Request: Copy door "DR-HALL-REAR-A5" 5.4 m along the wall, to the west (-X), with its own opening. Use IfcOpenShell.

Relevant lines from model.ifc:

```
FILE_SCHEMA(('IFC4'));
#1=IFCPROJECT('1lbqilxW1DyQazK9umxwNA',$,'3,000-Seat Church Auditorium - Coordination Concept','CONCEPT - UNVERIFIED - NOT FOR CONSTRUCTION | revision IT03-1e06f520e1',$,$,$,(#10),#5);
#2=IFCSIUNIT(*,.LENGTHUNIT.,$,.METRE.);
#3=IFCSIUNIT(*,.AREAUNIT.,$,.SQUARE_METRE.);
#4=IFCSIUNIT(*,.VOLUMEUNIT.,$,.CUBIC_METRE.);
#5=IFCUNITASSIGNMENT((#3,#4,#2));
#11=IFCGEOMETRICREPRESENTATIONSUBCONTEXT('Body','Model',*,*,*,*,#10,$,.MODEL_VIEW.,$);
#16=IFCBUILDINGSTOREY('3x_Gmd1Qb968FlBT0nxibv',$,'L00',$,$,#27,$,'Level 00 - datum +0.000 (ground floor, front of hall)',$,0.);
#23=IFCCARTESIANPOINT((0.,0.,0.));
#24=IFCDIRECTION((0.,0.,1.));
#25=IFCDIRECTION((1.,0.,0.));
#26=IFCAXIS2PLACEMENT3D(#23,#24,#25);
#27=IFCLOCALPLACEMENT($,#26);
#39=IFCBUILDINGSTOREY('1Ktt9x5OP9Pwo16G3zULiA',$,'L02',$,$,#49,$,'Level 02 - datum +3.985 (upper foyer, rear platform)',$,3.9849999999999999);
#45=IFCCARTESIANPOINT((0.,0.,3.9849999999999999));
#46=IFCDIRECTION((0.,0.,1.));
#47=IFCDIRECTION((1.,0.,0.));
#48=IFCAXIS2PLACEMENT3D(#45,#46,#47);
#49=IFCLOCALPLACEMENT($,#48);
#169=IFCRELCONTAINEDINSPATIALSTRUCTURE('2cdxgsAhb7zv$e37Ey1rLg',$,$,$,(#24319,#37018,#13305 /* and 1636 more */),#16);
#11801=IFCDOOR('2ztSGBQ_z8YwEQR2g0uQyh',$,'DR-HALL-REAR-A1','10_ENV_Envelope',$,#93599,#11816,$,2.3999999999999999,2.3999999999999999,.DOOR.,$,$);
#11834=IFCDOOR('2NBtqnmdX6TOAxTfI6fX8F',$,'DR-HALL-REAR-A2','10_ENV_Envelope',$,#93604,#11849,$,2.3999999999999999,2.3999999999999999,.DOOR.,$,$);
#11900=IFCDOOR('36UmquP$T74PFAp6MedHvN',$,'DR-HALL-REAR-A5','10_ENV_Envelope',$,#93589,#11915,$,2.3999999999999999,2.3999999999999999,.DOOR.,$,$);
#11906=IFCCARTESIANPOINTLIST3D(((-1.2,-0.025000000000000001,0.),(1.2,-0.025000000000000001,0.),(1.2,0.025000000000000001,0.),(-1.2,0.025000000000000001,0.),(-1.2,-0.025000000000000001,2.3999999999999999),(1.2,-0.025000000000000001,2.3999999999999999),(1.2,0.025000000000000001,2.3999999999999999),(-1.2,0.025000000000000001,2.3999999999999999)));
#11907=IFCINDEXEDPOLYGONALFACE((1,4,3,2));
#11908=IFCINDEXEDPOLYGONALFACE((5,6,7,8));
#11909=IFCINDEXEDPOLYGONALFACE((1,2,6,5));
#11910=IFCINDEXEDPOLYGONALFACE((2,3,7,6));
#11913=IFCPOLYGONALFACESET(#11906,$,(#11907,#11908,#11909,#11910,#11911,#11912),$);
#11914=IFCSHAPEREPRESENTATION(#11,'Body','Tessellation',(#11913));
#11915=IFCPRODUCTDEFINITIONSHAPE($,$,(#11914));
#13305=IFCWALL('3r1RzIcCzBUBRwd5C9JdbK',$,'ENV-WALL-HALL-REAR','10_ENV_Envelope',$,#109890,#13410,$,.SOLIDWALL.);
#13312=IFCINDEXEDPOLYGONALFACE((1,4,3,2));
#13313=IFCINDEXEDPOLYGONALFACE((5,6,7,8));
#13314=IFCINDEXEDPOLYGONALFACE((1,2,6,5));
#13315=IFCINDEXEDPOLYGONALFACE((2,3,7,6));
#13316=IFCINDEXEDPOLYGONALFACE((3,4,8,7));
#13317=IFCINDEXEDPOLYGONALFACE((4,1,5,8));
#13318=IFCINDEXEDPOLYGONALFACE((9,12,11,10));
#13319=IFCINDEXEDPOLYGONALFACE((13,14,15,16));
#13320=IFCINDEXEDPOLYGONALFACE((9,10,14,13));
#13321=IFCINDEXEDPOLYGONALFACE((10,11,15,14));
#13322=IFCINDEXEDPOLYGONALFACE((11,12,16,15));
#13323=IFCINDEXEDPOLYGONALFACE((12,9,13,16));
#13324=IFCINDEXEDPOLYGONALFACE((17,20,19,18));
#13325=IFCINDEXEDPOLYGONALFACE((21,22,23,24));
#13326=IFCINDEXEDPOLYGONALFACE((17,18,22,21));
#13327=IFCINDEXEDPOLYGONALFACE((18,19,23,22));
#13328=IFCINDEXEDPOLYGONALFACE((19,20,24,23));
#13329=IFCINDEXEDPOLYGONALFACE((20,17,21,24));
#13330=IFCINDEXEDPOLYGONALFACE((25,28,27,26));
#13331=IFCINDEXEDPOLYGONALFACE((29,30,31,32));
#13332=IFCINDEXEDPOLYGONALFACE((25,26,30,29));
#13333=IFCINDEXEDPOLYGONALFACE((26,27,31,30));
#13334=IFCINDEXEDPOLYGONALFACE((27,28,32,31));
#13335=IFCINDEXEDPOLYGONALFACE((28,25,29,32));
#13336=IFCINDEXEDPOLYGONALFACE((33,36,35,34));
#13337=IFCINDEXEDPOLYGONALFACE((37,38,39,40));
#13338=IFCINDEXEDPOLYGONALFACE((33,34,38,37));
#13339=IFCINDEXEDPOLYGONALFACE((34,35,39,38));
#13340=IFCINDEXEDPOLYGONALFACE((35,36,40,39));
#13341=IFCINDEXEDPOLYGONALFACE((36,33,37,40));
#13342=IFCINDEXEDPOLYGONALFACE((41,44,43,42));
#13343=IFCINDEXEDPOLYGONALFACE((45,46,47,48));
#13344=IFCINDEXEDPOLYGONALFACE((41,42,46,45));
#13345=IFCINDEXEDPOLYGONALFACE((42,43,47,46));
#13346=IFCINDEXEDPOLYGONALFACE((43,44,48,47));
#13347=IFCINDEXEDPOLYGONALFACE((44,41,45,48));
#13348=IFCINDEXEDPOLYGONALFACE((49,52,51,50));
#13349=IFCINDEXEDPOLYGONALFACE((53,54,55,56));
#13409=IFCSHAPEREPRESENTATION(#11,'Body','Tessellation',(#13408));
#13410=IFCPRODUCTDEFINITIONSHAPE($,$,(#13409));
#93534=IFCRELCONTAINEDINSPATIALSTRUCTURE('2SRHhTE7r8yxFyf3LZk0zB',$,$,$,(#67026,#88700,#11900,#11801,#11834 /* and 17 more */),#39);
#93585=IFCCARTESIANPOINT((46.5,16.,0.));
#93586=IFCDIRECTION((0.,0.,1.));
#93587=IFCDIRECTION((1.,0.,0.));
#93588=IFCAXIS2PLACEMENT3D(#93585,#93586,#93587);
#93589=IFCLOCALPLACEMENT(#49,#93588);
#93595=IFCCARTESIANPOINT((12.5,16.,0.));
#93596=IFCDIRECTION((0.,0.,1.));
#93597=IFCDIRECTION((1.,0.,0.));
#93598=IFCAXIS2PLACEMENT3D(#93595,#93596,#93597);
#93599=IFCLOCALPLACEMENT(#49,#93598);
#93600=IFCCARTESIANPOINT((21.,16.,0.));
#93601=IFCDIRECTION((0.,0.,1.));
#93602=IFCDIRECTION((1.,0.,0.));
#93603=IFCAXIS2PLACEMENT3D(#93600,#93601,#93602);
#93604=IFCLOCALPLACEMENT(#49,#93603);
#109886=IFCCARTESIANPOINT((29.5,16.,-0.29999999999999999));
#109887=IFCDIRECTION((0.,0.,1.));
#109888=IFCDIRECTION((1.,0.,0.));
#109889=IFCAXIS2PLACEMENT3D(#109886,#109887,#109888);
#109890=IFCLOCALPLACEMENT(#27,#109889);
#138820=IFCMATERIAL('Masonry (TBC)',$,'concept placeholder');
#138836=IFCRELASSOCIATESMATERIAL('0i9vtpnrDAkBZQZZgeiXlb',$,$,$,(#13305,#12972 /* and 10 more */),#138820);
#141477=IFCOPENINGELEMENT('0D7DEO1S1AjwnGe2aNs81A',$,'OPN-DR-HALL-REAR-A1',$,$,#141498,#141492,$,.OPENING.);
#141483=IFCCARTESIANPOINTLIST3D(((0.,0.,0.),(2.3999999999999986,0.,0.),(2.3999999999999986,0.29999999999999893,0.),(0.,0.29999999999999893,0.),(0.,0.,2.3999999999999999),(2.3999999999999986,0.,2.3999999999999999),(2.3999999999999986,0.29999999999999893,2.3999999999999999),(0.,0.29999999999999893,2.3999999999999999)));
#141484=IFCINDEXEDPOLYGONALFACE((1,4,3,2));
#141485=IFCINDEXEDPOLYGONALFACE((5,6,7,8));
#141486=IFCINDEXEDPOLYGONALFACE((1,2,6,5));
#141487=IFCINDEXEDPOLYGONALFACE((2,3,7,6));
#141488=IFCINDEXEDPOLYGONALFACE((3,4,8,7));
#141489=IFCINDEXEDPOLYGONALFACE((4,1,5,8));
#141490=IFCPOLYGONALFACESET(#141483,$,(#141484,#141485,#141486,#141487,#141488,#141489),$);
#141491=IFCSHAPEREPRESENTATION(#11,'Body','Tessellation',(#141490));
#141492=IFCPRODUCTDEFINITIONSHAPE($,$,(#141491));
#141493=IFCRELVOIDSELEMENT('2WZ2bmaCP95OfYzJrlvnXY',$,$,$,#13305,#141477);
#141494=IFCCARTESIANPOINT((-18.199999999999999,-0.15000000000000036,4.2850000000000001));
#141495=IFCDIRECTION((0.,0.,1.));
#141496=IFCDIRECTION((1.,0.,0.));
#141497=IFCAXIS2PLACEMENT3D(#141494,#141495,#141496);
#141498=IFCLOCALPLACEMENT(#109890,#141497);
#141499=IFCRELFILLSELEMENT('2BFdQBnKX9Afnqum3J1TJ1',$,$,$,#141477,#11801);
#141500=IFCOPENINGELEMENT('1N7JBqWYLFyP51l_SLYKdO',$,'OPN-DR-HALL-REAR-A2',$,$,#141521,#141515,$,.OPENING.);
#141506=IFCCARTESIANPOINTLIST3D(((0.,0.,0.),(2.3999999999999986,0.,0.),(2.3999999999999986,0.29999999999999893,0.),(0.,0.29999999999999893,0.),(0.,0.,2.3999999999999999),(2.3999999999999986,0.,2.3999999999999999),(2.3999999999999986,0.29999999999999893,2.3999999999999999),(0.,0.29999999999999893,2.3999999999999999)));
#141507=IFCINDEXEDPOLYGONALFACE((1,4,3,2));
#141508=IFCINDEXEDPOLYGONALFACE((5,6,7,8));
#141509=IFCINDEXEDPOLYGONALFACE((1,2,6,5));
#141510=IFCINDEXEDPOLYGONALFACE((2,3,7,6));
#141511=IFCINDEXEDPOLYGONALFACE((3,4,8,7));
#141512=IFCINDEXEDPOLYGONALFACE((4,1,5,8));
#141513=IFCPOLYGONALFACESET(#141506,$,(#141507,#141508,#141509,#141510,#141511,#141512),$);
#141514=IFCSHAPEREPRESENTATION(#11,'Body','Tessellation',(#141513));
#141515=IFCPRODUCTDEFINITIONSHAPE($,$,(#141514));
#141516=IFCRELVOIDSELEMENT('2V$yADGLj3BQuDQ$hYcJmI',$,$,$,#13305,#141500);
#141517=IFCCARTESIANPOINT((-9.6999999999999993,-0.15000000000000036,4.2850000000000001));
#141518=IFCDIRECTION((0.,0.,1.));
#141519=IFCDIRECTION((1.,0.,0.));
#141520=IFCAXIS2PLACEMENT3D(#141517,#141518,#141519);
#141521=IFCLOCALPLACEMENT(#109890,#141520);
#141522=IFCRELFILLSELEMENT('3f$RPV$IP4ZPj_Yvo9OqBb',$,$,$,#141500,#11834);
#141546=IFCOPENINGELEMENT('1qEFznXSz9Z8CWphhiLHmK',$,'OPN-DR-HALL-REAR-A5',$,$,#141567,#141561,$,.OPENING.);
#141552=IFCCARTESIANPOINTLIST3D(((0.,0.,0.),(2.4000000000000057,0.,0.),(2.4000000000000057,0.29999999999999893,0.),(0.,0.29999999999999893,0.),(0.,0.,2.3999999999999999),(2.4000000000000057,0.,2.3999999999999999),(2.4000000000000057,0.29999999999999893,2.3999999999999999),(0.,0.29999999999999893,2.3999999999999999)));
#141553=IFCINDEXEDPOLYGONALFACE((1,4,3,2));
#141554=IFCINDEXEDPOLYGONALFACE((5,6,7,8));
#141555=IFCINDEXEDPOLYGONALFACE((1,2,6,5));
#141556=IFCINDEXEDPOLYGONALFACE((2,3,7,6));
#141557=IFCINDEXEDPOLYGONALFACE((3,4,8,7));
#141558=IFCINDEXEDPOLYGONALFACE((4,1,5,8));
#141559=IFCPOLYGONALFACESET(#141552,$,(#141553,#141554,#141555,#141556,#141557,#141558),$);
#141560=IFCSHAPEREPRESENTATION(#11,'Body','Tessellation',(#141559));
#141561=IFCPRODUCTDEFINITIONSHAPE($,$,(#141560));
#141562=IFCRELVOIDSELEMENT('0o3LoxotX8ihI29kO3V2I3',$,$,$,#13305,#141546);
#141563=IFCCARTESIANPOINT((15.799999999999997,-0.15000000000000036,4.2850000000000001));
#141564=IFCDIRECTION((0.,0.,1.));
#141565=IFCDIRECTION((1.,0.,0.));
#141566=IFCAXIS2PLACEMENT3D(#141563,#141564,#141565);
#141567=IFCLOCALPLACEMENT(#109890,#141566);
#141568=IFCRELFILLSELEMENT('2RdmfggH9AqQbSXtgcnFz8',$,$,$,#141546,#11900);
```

```python
import ifcopenshell
import ifcopenshell.api.feature
import ifcopenshell.api.geometry
import ifcopenshell.api.root
import ifcopenshell.geom
import ifcopenshell.util.element
import ifcopenshell.util.placement
import ifcopenshell.util.shape
import ifcopenshell.util.unit

model = ifcopenshell.open("model.ifc")
unit_scale = ifcopenshell.util.unit.calculate_unit_scale(model)
settings = ifcopenshell.geom.settings()


def volume(element):
    """Net volume in cubic metres, openings subtracted."""
    shape = ifcopenshell.geom.create_shape(settings, element)
    return ifcopenshell.util.shape.get_volume(shape.geometry)


door = model.by_guid("36UmquP$T74PFAp6MedHvN")
opening = door.FillsVoids[0].RelatingOpeningElement
wall = opening.VoidsElements[0].RelatingBuildingElement
before = volume(wall)
shift = ifcopenshell.util.placement.get_local_placement(wall.ObjectPlacement)[:3, 0] * -5.4 / unit_scale

# copy_class copies the void relationship, type, container and properties, but no geometry.
new_opening = ifcopenshell.api.root.copy_class(model, product=opening)
new_opening.Representation = ifcopenshell.util.element.copy_deep(
    model, opening.Representation, exclude=["IfcGeometricRepresentationContext", "IfcRepresentationMap"]
)
new_door = ifcopenshell.api.root.copy_class(model, product=door)
new_door.Representation = ifcopenshell.util.element.copy_deep(
    model, door.Representation, exclude=["IfcGeometricRepresentationContext", "IfcRepresentationMap"]
)
ifcopenshell.api.feature.add_filling(model, opening=new_opening, element=new_door)

for old, new in ((opening, new_opening), (door, new_door)):
    matrix = ifcopenshell.util.placement.get_local_placement(old.ObjectPlacement)
    matrix[:3, 3] += shift
    ifcopenshell.api.geometry.edit_object_placement(model, product=new, matrix=matrix, is_si=False)

after = volume(wall)

print(f"wall volume {before:.3f} -> {after:.3f} m3")

model.write("model_rev.ifc")
```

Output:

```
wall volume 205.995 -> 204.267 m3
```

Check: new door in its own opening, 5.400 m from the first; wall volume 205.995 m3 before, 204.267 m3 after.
